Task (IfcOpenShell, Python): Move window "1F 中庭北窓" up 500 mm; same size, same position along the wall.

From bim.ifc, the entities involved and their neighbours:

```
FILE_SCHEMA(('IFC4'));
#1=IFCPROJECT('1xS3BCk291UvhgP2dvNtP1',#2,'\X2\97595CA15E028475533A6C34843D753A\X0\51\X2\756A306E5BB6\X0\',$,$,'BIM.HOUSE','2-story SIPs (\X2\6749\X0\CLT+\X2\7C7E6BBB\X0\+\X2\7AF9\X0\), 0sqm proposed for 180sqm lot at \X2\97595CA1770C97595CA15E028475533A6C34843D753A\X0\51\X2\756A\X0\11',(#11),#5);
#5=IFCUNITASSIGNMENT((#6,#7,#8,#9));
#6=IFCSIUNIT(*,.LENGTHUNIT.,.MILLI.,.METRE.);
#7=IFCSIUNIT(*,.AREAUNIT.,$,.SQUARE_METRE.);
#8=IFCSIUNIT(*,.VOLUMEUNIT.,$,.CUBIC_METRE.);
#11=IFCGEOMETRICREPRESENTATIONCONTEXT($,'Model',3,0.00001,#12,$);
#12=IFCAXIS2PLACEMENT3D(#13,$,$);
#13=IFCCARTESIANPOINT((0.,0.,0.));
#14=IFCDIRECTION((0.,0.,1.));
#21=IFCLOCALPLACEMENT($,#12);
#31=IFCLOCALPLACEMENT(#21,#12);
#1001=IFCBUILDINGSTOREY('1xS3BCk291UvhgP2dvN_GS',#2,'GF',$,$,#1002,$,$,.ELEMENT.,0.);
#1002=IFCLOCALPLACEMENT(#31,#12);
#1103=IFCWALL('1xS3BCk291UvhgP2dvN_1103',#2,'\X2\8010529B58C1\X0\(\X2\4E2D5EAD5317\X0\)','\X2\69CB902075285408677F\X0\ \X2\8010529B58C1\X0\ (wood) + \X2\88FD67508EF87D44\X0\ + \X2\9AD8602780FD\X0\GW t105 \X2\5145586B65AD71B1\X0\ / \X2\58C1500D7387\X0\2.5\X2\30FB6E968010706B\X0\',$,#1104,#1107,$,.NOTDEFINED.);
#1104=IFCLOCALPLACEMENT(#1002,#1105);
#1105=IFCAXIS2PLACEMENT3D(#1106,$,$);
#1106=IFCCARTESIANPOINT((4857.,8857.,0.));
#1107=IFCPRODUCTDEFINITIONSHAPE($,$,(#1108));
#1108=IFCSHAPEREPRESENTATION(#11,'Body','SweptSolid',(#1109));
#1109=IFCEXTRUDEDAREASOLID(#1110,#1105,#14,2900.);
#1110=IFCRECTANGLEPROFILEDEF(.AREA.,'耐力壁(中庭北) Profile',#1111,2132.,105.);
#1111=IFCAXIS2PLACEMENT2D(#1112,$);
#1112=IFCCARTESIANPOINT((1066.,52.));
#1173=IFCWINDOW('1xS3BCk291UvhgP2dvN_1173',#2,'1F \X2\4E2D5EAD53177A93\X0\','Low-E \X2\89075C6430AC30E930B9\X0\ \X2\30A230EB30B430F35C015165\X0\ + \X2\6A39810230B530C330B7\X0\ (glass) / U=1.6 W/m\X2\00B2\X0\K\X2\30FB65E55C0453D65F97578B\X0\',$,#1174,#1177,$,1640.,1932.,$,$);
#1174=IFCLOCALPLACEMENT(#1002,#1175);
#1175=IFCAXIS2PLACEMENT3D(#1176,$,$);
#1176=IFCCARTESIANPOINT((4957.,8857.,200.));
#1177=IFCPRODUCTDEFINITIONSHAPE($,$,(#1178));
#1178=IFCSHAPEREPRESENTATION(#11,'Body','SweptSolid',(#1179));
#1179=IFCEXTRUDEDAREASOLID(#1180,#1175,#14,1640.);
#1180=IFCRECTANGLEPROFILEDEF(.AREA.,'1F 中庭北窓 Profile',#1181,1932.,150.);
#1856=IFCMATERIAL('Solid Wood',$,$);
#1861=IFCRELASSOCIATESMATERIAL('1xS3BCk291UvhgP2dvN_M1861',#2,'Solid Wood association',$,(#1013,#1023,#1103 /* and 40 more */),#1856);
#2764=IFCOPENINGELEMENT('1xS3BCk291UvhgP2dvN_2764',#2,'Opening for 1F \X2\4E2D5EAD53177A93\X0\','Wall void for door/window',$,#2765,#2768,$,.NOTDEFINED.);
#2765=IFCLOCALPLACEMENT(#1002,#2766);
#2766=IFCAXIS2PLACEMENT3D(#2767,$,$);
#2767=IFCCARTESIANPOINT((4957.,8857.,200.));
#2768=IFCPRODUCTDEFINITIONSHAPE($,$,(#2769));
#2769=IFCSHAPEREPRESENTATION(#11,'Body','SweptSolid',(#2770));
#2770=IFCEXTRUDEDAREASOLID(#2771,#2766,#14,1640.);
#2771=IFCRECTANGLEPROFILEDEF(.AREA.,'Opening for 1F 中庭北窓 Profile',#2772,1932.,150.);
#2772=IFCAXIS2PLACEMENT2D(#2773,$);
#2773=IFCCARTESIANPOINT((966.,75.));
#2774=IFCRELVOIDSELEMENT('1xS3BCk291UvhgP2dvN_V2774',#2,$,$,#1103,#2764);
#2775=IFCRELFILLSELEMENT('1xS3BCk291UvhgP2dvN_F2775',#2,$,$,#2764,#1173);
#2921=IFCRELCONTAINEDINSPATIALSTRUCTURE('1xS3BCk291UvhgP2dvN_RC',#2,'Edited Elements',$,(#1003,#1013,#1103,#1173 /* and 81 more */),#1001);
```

```python
import numpy as np
import ifcopenshell
import ifcopenshell.api.geometry
import ifcopenshell.util.placement
import ifcopenshell.util.unit

model = ifcopenshell.open("bim.ifc")
unit_scale = ifcopenshell.util.unit.calculate_unit_scale(model)

window = model.by_id(1173)
opening = window.FillsVoids[0].RelatingOpeningElement
dz = 0.5 / unit_scale

shift = np.array([0.0, 0.0, dz])
# The window is not placed relative to its opening, so move both.
for product in (opening, window):
    matrix = ifcopenshell.util.placement.get_local_placement(product.ObjectPlacement)
    matrix[:3, 3] += shift
    ifcopenshell.api.geometry.edit_object_placement(model, product=product, matrix=matrix, is_si=False)

print(f"moved by {dz * unit_scale:+.3f} m")

model.write("bim_edited.ifc")
```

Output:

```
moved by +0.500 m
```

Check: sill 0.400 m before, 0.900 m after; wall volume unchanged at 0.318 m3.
